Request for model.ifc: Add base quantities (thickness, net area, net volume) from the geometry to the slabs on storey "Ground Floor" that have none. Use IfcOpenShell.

First a look at what the model holds.

```python
import ifcopenshell
import ifcopenshell.util.element
import ifcopenshell.util.unit

model = ifcopenshell.open("model.ifc")
print(model.schema)
for unit_type in ("LENGTHUNIT", "AREAUNIT", "VOLUMEUNIT"):
    print(unit_type, ifcopenshell.util.unit.calculate_unit_scale(model, unit_type))
storey = next(s for s in model.by_type("IfcBuildingStorey") if s.Name == "Ground Floor")
slabs = [e for e in ifcopenshell.util.element.get_decomposition(storey) if e.is_a("IfcSlab")]
for e in sorted(slabs, key=lambda e: e.id()):
    print(e.id(), e.is_a(), e.Name, list(ifcopenshell.util.element.get_psets(e, qtos_only=True)), sep=" | ")
```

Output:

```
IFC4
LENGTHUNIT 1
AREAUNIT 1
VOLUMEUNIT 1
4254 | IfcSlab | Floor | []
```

```python
import ifcopenshell
import ifcopenshell.api.pset
import ifcopenshell.geom
import ifcopenshell.util.element
import ifcopenshell.util.shape
import ifcopenshell.util.unit

model = ifcopenshell.open("model.ifc")
unit_scale = ifcopenshell.util.unit.calculate_unit_scale(model)
area_scale = ifcopenshell.util.unit.calculate_unit_scale(model, "AREAUNIT")
volume_scale = ifcopenshell.util.unit.calculate_unit_scale(model, "VOLUMEUNIT")
settings = ifcopenshell.geom.settings()

storey = next(s for s in model.by_type("IfcBuildingStorey") if s.Name == "Ground Floor")
slabs = [e for e in ifcopenshell.util.element.get_decomposition(storey) if e.is_a("IfcSlab")]

for e in sorted(slabs, key=lambda e: e.id()):
    if ifcopenshell.util.element.get_psets(e, qtos_only=True, should_inherit=False):
        continue
    # Geometry comes back in metres, in the element's own axes.
    shape = ifcopenshell.geom.create_shape(settings, e)
    values = {
        "Width": ifcopenshell.util.shape.get_z(shape.geometry) / unit_scale,
        "NetArea": ifcopenshell.util.shape.get_footprint_area(shape.geometry) / area_scale,
        "NetVolume": ifcopenshell.util.shape.get_volume(shape.geometry) / volume_scale,
    }
    qto = ifcopenshell.api.pset.add_qto(model, product=e, name="Qto_SlabBaseQuantities")
    ifcopenshell.api.pset.edit_qto(model, qto=qto, properties=values)
    print(e.id(), {k: round(v, 3) for k, v in values.items()})

model.write("model-out.ifc")
```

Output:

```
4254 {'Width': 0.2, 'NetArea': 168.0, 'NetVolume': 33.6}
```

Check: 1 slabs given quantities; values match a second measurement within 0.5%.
